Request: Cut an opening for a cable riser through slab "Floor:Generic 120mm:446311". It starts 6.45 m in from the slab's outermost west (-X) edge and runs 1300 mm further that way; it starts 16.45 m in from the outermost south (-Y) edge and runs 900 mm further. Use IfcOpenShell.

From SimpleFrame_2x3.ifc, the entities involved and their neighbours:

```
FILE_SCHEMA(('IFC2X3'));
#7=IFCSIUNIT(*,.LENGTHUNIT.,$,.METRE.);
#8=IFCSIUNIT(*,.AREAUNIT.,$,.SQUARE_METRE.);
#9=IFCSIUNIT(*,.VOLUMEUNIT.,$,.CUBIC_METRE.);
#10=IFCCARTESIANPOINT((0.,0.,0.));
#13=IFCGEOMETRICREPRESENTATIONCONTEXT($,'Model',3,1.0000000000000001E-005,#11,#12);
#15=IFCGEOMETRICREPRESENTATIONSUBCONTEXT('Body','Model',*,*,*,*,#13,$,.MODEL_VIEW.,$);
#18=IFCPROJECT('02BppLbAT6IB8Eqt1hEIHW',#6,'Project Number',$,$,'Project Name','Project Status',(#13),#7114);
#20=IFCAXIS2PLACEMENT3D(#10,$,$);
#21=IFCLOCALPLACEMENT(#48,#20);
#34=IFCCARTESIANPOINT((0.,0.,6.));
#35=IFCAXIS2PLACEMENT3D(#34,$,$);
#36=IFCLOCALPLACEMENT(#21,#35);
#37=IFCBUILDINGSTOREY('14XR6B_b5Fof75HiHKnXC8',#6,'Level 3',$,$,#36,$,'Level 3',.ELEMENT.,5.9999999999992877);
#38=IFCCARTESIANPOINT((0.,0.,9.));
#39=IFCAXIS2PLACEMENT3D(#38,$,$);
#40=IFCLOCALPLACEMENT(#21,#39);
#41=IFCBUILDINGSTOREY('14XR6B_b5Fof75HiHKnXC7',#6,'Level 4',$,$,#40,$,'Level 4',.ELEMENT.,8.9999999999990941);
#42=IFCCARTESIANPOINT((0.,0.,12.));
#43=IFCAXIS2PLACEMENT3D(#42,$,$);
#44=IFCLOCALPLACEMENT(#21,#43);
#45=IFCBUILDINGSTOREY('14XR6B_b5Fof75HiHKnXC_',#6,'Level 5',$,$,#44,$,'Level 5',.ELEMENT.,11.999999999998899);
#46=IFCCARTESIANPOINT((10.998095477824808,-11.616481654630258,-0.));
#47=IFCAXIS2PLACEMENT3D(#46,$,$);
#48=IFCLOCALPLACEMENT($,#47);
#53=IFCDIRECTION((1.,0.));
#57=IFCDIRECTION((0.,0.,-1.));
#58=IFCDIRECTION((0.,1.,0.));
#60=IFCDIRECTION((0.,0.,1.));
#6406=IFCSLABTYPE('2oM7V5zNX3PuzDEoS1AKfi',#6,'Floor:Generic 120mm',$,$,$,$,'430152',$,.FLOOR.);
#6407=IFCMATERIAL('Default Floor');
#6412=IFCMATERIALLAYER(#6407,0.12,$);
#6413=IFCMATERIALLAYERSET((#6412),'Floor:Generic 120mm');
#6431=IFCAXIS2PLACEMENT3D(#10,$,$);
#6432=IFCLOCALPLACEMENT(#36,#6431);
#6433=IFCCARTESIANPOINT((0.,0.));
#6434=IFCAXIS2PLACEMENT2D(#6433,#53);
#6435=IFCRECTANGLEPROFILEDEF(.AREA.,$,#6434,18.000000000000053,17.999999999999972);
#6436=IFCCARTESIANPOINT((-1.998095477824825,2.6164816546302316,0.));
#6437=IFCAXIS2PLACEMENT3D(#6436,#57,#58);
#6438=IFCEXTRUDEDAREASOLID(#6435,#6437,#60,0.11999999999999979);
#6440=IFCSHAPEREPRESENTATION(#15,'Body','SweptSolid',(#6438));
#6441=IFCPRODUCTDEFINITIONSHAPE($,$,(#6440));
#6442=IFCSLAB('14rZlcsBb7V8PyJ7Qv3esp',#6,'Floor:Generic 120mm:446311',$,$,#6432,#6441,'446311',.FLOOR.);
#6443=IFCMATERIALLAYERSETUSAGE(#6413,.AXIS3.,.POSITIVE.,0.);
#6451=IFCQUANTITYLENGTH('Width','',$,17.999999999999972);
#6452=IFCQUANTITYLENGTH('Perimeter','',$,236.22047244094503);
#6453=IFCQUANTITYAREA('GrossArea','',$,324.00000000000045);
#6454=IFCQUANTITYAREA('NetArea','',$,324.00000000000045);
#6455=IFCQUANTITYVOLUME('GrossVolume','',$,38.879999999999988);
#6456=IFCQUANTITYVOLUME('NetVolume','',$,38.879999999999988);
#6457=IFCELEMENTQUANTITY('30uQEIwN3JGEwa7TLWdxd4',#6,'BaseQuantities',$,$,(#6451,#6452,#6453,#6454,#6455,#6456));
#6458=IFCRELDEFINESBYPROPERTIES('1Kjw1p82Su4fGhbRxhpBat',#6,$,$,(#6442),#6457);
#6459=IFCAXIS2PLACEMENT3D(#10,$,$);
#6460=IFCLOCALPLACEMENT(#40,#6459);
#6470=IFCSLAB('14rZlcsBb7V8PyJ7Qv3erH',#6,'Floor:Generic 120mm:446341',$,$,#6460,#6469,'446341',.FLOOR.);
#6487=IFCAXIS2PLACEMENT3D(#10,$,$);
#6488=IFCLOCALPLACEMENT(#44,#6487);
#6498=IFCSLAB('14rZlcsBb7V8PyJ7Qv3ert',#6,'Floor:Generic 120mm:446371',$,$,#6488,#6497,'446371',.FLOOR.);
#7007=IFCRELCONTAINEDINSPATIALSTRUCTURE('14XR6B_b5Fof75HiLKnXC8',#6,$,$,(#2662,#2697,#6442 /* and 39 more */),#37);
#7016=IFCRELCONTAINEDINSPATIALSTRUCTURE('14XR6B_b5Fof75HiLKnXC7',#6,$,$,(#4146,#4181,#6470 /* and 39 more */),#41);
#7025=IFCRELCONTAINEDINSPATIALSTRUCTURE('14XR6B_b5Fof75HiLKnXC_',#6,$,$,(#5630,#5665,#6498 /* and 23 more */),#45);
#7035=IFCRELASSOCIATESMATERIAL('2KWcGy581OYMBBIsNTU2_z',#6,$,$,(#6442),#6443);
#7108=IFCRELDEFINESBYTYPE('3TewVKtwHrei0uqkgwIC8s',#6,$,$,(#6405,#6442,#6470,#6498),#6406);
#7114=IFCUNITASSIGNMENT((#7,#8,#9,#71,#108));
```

```python
import numpy as np
import ifcopenshell
import ifcopenshell.api.feature
import ifcopenshell.api.geometry
import ifcopenshell.api.pset
import ifcopenshell.api.root
import ifcopenshell.geom
import ifcopenshell.util.element
import ifcopenshell.util.placement
import ifcopenshell.util.representation
import ifcopenshell.util.shape
import ifcopenshell.util.unit

model = ifcopenshell.open("SimpleFrame_2x3.ifc")
unit_scale = ifcopenshell.util.unit.calculate_unit_scale(model)
area_scale = ifcopenshell.util.unit.calculate_unit_scale(model, "AREAUNIT")
volume_scale = ifcopenshell.util.unit.calculate_unit_scale(model, "VOLUMEUNIT")
settings = ifcopenshell.geom.settings()


def volume(element):
    """Net volume in cubic metres, openings subtracted."""
    shape = ifcopenshell.geom.create_shape(settings, element)
    return ifcopenshell.util.shape.get_volume(shape.geometry)


slab = model.by_id(6442)
before = volume(slab)

# Extent in the slab's own axes, in metres. The edges named are its -X and -Y sides.
slab_shape = ifcopenshell.geom.create_shape(settings, slab)
vertices = ifcopenshell.util.shape.get_vertices(slab_shape.geometry)
x_min, y_min, bottom = vertices.min(axis=0)
top = vertices[:, 2].max()

opening = ifcopenshell.api.root.create_entity(model, ifc_class="IfcOpeningElement", name="Cable riser opening")
context = ifcopenshell.util.representation.get_context(model, "Model", "Body", "MODEL_VIEW")
width, depth = 1.3, 0.9
outline = [(0.0, 0.0), (width, 0.0), (width, depth), (0.0, depth), (0.0, 0.0)]
# Overshoot both faces by 50 mm so the cut is clean.
shape = ifcopenshell.api.geometry.add_slab_representation(
    model, context=context, depth=top - bottom + 0.1, polyline=outline
)
ifcopenshell.api.geometry.assign_representation(model, product=opening, representation=shape)

matrix = ifcopenshell.util.placement.get_local_placement(slab.ObjectPlacement)
matrix[:, 3] = matrix @ np.append(np.array([x_min + 6.45, y_min + 16.45, bottom - 0.05]) / unit_scale, 1.0)
ifcopenshell.api.geometry.edit_object_placement(model, product=opening, matrix=matrix, is_si=False)
ifcopenshell.api.feature.add_feature(model, feature=opening, element=slab)

after = volume(slab)

# Update the slab's stored quantities.
qto = model.by_id(ifcopenshell.util.element.get_pset(slab, "BaseQuantities", should_inherit=False)["id"])
ifcopenshell.api.pset.edit_qto(model, qto=qto, properties={
    "NetArea": after / (top - bottom) / area_scale,
    "NetVolume": after / volume_scale,
})

print(f"slab volume {before:.3f} -> {after:.3f} m3")

model.write("SimpleFrame_2x3_rev.ifc")
```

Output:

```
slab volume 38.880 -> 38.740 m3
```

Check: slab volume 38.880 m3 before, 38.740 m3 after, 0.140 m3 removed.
